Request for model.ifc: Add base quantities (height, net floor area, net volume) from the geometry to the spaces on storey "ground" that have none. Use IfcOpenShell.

First a look at what the model holds.

```python
import ifcopenshell
import ifcopenshell.util.element
import ifcopenshell.util.unit

model = ifcopenshell.open("model.ifc")
print(model.schema)
for unit_type in ("LENGTHUNIT", "AREAUNIT", "VOLUMEUNIT"):
    print(unit_type, ifcopenshell.util.unit.calculate_unit_scale(model, unit_type))
storey = next(s for s in model.by_type("IfcBuildingStorey") if s.Name == "ground")
spaces = [e for e in ifcopenshell.util.element.get_decomposition(storey) if e.is_a("IfcSpace")]
for e in sorted(spaces, key=lambda e: e.id()):
    print(e.id(), e.is_a(), e.Name, list(ifcopenshell.util.element.get_psets(e, qtos_only=True)), sep=" | ")
```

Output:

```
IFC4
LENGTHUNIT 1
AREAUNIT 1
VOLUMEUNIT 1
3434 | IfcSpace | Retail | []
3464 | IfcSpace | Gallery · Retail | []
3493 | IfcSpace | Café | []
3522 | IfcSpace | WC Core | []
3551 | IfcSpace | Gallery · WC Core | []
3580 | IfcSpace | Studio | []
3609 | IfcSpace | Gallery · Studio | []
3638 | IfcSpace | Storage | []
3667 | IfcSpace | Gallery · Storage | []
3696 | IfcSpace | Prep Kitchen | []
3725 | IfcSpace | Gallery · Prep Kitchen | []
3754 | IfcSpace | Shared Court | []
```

```python
import ifcopenshell
import ifcopenshell.api.pset
import ifcopenshell.geom
import ifcopenshell.util.element
import ifcopenshell.util.shape
import ifcopenshell.util.unit

model = ifcopenshell.open("model.ifc")
unit_scale = ifcopenshell.util.unit.calculate_unit_scale(model)
area_scale = ifcopenshell.util.unit.calculate_unit_scale(model, "AREAUNIT")
volume_scale = ifcopenshell.util.unit.calculate_unit_scale(model, "VOLUMEUNIT")
settings = ifcopenshell.geom.settings()

storey = next(s for s in model.by_type("IfcBuildingStorey") if s.Name == "ground")
spaces = [e for e in ifcopenshell.util.element.get_decomposition(storey) if e.is_a("IfcSpace")]

for e in sorted(spaces, key=lambda e: e.id()):
    if ifcopenshell.util.element.get_psets(e, qtos_only=True, should_inherit=False):
        continue
    # Geometry comes back in metres, in the element's own axes.
    shape = ifcopenshell.geom.create_shape(settings, e)
    values = {
        "Height": ifcopenshell.util.shape.get_z(shape.geometry) / unit_scale,
        "NetFloorArea": ifcopenshell.util.shape.get_footprint_area(shape.geometry) / area_scale,
        "NetVolume": ifcopenshell.util.shape.get_volume(shape.geometry) / volume_scale,
    }
    qto = ifcopenshell.api.pset.add_qto(model, product=e, name="Qto_SpaceBaseQuantities")
    ifcopenshell.api.pset.edit_qto(model, qto=qto, properties=values)
    print(e.id(), {k: round(v, 3) for k, v in values.items()})

model.write("model_edited.ifc")
```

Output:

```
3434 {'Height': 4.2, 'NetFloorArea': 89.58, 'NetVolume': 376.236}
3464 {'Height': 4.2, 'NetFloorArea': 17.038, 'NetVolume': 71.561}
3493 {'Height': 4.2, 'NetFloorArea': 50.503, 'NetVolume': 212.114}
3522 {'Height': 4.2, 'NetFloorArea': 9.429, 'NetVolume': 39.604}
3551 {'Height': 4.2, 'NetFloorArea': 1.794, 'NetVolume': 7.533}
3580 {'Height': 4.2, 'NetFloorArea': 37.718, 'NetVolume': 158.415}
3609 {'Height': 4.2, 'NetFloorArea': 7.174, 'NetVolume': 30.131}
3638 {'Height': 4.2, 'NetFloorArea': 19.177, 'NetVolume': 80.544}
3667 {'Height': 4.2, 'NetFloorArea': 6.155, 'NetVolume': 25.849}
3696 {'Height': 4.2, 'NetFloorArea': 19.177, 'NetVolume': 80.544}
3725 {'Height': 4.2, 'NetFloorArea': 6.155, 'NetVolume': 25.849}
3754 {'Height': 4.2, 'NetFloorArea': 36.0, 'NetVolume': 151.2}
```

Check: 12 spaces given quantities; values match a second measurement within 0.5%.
